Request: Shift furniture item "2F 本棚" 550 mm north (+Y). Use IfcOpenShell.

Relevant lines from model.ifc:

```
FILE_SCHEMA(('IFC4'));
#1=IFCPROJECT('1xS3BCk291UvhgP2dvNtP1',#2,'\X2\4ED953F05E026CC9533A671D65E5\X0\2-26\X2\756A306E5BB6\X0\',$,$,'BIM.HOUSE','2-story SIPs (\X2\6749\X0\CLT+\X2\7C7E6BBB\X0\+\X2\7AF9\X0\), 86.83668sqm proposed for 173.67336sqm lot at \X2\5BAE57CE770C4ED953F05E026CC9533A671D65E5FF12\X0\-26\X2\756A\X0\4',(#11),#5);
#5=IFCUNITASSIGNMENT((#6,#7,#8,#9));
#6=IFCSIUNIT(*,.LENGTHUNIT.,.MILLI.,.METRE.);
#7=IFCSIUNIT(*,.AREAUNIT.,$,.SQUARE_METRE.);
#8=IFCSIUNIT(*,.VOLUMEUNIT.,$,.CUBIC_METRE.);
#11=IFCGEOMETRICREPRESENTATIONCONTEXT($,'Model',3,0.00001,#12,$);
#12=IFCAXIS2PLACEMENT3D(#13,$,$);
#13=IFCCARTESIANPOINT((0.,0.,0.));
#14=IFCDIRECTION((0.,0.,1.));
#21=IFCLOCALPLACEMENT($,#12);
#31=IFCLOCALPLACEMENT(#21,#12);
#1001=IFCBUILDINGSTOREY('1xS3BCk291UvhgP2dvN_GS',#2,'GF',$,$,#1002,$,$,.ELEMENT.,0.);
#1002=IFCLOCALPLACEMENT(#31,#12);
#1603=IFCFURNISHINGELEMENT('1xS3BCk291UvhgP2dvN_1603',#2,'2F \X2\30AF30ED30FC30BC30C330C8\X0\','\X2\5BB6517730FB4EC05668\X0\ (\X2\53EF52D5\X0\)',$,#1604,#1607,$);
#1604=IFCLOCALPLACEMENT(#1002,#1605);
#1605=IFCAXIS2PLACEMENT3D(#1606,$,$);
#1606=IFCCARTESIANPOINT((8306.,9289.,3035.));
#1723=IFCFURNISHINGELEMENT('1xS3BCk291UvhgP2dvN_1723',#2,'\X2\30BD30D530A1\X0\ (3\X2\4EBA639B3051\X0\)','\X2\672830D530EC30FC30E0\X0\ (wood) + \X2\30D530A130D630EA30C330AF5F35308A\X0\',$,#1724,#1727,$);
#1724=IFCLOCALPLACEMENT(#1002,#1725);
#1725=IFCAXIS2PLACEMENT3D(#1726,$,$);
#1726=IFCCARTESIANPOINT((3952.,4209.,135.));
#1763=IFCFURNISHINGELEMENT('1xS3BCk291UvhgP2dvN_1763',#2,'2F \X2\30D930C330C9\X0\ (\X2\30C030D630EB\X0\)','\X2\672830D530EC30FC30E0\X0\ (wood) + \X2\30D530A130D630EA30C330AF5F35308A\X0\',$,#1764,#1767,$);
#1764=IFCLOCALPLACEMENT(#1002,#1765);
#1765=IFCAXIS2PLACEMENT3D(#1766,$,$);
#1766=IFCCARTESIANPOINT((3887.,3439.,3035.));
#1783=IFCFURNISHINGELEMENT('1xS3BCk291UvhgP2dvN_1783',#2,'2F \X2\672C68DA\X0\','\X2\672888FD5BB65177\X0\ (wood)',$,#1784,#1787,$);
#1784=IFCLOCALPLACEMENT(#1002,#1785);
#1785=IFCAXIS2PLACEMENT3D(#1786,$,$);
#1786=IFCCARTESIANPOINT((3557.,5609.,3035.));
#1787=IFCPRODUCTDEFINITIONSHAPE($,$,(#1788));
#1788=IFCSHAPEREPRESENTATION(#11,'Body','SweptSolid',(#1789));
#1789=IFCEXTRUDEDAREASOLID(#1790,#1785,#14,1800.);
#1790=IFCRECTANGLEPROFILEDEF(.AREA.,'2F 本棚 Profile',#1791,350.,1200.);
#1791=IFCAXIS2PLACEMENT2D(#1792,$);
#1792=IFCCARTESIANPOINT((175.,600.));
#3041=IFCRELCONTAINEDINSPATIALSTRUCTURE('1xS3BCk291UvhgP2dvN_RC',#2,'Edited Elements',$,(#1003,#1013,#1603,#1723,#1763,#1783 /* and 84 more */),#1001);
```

```python
import ifcopenshell
import ifcopenshell.api.geometry
import ifcopenshell.util.placement

model = ifcopenshell.open("model.ifc")

item = model.by_id(1783)
matrix = ifcopenshell.util.placement.get_local_placement(item.ObjectPlacement)
matrix[1, 3] += 550.0
ifcopenshell.api.geometry.edit_object_placement(model, product=item, matrix=matrix, is_si=False)

print(ifcopenshell.util.placement.get_local_placement(item.ObjectPlacement).round(3) + 0.0)

model.write("model-out.ifc")
```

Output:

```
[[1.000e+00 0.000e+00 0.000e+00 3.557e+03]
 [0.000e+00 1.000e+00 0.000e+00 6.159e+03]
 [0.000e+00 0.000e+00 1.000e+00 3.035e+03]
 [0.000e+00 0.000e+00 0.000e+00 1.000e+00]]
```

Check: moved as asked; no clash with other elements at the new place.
